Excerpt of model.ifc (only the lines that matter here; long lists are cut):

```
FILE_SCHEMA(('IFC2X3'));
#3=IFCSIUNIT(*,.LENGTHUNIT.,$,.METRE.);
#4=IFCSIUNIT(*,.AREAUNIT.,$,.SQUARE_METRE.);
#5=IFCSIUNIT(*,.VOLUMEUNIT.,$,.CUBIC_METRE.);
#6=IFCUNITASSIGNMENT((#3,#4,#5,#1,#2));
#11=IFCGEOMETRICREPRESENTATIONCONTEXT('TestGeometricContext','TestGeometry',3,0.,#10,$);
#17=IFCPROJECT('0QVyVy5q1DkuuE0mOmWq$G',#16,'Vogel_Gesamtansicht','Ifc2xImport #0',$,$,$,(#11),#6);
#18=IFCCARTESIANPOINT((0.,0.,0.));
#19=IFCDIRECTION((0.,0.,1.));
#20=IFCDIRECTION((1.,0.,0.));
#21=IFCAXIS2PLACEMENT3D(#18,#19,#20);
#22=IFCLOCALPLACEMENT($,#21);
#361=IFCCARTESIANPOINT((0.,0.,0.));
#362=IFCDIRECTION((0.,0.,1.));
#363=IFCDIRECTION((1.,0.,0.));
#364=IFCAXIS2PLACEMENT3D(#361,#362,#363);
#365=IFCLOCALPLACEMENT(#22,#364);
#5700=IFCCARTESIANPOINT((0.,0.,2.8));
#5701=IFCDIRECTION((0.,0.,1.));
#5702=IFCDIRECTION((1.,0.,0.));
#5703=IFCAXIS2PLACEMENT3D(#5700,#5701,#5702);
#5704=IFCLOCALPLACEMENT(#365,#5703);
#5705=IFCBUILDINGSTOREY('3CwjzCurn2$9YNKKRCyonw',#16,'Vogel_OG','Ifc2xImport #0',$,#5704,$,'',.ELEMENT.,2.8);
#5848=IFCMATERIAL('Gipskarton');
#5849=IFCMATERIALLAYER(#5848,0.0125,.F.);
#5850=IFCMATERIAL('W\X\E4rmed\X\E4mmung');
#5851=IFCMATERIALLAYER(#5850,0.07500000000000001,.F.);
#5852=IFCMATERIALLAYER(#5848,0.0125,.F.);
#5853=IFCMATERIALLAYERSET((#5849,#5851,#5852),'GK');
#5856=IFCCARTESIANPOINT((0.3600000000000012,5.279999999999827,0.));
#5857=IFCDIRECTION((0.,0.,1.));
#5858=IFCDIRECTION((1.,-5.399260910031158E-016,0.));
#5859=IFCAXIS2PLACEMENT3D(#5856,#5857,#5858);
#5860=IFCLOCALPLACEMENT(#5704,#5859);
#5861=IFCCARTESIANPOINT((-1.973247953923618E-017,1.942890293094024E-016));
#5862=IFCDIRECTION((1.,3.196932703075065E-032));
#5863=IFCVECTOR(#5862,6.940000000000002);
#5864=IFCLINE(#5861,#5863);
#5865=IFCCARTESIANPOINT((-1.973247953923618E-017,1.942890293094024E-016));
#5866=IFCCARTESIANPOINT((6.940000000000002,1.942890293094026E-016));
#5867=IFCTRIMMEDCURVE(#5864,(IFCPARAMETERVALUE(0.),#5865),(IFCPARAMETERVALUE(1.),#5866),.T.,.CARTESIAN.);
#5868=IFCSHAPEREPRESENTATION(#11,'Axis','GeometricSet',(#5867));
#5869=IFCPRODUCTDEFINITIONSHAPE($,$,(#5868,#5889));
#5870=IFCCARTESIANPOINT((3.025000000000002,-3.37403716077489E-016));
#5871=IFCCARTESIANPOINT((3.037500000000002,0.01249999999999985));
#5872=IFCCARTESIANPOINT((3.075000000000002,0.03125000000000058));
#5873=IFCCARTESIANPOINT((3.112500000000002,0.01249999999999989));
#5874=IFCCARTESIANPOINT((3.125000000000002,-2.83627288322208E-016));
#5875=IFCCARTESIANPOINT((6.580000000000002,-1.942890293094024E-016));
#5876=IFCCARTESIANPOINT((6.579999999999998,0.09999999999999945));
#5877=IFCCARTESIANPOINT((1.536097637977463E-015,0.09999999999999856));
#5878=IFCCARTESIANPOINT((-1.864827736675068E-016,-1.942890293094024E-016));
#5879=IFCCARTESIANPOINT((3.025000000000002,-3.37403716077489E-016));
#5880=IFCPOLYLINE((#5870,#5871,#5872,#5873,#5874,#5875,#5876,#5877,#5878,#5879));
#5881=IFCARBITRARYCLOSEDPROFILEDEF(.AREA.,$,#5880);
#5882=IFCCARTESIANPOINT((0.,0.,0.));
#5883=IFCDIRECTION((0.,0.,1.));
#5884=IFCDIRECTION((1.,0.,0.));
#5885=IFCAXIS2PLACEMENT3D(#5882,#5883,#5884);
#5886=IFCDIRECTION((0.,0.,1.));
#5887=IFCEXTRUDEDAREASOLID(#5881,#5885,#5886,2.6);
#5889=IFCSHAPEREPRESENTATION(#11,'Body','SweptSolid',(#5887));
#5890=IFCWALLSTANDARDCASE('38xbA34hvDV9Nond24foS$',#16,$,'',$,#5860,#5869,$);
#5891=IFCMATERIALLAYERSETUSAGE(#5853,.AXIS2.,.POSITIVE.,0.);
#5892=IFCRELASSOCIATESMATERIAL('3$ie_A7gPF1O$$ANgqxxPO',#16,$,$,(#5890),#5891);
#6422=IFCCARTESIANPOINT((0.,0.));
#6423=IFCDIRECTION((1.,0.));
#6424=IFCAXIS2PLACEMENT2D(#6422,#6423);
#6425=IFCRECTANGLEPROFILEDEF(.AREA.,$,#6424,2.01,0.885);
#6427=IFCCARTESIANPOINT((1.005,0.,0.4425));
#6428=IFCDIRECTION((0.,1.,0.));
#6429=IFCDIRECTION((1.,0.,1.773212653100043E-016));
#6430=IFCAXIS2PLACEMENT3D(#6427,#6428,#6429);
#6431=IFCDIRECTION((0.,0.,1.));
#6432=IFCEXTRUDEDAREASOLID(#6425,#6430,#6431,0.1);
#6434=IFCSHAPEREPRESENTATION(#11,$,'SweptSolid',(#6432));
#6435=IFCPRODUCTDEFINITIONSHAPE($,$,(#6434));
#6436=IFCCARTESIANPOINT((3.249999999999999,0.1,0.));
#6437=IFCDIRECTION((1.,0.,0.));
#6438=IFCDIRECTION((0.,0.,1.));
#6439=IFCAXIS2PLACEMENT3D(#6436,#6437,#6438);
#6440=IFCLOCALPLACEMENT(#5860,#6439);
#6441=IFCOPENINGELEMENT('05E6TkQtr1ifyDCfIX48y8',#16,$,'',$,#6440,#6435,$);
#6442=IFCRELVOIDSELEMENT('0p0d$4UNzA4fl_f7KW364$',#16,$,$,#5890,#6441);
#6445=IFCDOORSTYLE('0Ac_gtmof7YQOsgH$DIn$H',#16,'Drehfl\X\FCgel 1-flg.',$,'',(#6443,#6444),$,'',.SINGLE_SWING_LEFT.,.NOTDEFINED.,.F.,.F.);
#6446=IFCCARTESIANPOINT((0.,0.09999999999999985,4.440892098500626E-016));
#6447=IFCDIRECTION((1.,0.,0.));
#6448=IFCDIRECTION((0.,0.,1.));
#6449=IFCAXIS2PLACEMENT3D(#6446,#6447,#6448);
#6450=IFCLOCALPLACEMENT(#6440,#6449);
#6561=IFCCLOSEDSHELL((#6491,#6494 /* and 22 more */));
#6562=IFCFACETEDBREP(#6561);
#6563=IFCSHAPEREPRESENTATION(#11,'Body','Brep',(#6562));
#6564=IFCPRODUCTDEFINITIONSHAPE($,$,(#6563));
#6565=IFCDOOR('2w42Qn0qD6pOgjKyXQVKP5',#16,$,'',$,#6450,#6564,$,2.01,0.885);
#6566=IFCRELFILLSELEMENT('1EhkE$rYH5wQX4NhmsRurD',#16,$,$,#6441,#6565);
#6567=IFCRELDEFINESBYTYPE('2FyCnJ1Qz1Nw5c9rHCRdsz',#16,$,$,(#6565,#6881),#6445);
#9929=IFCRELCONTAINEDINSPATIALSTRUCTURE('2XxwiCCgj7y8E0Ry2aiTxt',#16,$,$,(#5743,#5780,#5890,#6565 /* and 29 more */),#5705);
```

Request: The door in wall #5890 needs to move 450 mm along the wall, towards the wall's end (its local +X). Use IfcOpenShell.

```python
import ifcopenshell
import ifcopenshell.api.geometry
import ifcopenshell.util.placement

model = ifcopenshell.open("model.ifc")

door = model.by_guid("2w42Qn0qD6pOgjKyXQVKP5")
opening = door.FillsVoids[0].RelatingOpeningElement
wall = opening.VoidsElements[0].RelatingBuildingElement

wall_matrix = ifcopenshell.util.placement.get_local_placement(wall.ObjectPlacement)
shift = wall_matrix[:3, 0] * 0.45
before = ifcopenshell.util.placement.get_local_placement(door.ObjectPlacement)[:3, 3].copy()

# The door is placed relative to its opening, so it follows when the opening moves.
matrix = ifcopenshell.util.placement.get_local_placement(opening.ObjectPlacement)
matrix[:3, 3] += shift
ifcopenshell.api.geometry.edit_object_placement(
    model, product=opening, matrix=matrix, is_si=False, should_transform_children=True
)

after = ifcopenshell.util.placement.get_local_placement(door.ObjectPlacement)[:3, 3]
print("door moved by", (after - before).round(3) + 0.0)

model.write("model-out.ifc")
```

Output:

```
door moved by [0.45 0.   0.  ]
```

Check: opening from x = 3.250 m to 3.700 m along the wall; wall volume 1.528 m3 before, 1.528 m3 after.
